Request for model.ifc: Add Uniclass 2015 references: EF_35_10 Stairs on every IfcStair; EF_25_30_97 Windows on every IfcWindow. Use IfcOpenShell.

First a look at what the model holds.

```python
import ifcopenshell

model = ifcopenshell.open("model.ifc")
print(model.schema)
print("classifications:", [c.Name for c in model.by_type("IfcClassification")])
for ifc_class in ("IfcDoor", "IfcRoof", "IfcStair", "IfcWall", "IfcWindow"):
    print(ifc_class, len(model.by_type(ifc_class)))
```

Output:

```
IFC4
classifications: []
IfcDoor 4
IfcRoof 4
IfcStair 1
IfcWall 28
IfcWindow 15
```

```python
import ifcopenshell
import ifcopenshell.api.classification

model = ifcopenshell.open("model.ifc")

system = ifcopenshell.api.classification.add_classification(model, classification="Uniclass 2015")

codes = {
    "IfcStair": ("EF_35_10", "Stairs"),
    "IfcWindow": ("EF_25_30_97", "Windows"),
}
for ifc_class, (code, name) in codes.items():
    products = model.by_type(ifc_class)
    ifcopenshell.api.classification.add_reference(
        model, products=products, classification=system, identification=code, name=name
    )
    print(code, len(products))

model.write("model_v2.ifc")
```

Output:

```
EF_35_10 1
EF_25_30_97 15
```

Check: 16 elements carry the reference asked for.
